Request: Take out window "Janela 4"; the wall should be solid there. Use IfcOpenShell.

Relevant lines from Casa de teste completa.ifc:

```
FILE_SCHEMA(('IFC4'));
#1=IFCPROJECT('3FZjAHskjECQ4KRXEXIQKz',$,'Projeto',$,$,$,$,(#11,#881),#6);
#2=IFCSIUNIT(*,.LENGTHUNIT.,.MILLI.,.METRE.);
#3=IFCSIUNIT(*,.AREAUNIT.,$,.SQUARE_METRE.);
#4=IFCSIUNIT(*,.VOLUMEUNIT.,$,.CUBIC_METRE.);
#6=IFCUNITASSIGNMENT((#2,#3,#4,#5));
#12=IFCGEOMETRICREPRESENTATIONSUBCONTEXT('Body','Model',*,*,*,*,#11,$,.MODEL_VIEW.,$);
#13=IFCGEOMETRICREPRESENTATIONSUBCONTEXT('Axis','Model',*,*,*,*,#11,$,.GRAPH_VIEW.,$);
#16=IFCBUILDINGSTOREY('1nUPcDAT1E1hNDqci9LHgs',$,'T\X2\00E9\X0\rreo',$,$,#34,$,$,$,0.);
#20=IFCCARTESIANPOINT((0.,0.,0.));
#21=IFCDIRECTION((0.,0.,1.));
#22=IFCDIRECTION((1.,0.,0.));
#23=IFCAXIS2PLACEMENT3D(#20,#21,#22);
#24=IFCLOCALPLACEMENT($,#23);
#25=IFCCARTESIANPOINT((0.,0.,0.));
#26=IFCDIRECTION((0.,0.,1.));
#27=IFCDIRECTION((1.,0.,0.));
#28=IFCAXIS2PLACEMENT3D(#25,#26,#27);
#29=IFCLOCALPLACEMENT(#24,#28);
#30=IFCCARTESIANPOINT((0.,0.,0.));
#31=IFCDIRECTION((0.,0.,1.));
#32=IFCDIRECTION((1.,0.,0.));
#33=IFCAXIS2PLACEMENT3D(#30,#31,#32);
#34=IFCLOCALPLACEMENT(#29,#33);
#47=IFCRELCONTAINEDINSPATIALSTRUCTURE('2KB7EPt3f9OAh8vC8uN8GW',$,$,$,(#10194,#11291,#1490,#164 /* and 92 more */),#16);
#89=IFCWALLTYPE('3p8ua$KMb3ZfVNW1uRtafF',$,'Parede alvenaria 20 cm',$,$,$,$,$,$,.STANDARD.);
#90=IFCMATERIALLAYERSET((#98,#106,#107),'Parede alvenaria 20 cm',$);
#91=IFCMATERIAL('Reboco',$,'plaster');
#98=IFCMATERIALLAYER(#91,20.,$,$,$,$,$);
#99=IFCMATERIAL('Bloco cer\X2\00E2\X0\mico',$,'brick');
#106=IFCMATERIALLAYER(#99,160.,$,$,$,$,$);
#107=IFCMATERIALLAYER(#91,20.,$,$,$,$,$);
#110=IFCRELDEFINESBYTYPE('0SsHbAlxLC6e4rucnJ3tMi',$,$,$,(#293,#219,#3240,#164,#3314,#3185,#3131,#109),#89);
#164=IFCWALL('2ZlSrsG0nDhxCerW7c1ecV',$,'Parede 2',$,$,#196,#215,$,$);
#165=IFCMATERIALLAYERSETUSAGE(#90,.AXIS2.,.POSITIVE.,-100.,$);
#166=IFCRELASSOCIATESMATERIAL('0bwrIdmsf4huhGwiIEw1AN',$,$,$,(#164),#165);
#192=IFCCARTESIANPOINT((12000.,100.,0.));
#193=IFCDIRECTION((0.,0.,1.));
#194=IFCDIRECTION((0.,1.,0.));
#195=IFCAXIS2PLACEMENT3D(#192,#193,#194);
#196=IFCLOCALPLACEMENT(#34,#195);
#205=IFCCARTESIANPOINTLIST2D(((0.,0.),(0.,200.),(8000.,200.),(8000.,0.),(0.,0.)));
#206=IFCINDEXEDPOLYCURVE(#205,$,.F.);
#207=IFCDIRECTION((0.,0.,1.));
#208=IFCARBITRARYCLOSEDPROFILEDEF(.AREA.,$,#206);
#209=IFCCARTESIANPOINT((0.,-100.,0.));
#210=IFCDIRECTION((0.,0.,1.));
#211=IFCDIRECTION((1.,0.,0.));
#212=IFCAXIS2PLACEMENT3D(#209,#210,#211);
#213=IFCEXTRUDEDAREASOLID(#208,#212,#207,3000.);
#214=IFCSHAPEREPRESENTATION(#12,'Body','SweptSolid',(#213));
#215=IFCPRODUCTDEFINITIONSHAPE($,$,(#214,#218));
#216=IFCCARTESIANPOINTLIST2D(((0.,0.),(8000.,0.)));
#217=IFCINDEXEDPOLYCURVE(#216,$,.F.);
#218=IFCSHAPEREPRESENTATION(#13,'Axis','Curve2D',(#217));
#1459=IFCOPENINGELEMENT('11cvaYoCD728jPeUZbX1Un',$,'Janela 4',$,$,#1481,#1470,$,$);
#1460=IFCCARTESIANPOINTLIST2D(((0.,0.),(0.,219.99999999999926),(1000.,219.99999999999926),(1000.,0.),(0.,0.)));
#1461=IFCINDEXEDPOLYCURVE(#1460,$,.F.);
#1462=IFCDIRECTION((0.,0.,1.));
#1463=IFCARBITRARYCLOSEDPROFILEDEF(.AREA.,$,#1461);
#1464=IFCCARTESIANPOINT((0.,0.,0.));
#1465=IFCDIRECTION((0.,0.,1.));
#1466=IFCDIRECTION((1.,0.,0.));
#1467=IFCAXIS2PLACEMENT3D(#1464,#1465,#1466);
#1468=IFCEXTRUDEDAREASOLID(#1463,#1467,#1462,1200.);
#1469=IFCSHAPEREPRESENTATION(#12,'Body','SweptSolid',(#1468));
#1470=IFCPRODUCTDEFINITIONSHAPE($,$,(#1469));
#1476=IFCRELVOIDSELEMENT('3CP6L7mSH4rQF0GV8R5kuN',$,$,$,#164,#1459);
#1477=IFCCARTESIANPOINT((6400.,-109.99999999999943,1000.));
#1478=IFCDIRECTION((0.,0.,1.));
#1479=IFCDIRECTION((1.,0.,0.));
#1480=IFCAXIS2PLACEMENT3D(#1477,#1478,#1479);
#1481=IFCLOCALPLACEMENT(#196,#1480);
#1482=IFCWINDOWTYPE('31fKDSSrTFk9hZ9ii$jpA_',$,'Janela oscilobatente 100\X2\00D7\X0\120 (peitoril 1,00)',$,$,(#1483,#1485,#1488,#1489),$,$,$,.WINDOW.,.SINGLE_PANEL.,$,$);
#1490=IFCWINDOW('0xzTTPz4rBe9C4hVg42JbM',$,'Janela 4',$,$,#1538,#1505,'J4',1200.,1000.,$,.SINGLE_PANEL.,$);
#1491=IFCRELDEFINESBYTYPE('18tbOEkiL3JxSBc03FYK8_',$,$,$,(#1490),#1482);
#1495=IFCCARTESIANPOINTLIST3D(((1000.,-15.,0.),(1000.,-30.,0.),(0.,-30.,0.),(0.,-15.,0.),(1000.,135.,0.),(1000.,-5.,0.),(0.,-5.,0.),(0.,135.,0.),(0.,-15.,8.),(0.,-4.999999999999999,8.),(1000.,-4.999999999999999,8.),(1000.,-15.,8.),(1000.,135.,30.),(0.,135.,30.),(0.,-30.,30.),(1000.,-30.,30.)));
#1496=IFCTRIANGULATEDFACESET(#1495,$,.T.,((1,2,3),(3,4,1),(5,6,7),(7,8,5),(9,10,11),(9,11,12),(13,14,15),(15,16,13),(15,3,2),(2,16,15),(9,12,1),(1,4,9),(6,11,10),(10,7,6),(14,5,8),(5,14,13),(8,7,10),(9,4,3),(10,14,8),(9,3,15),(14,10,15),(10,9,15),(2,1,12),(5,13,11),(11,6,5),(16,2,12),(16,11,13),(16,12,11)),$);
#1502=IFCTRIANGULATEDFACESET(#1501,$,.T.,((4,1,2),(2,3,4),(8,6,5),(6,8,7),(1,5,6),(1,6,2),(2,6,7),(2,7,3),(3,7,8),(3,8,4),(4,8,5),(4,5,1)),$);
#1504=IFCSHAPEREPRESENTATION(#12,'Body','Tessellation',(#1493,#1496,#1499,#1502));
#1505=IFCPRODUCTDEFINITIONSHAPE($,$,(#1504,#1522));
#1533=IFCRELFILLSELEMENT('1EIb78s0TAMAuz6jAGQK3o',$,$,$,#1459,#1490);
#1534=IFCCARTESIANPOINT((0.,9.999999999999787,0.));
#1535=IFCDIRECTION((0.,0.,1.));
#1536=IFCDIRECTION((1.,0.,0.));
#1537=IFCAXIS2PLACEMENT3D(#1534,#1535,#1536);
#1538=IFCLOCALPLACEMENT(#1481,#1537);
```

```python
import ifcopenshell
import ifcopenshell.api.feature
import ifcopenshell.api.root
import ifcopenshell.geom
import ifcopenshell.util.shape

model = ifcopenshell.open("Casa de teste completa.ifc")
settings = ifcopenshell.geom.settings()


def volume(element):
    """Net volume in cubic metres, openings subtracted."""
    shape = ifcopenshell.geom.create_shape(settings, element)
    return ifcopenshell.util.shape.get_volume(shape.geometry)


window = model.by_id(1490)
opening = window.FillsVoids[0].RelatingOpeningElement
wall = opening.VoidsElements[0].RelatingBuildingElement
before = volume(wall)

ifcopenshell.api.root.remove_product(model, product=window)
ifcopenshell.api.feature.remove_feature(model, feature=opening)

after = volume(wall)

print(f"wall volume {before:.3f} -> {after:.3f} m3")

model.write("Casa de teste completa-out.ifc")
```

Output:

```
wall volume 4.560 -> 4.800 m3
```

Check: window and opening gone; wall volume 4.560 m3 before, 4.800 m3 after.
